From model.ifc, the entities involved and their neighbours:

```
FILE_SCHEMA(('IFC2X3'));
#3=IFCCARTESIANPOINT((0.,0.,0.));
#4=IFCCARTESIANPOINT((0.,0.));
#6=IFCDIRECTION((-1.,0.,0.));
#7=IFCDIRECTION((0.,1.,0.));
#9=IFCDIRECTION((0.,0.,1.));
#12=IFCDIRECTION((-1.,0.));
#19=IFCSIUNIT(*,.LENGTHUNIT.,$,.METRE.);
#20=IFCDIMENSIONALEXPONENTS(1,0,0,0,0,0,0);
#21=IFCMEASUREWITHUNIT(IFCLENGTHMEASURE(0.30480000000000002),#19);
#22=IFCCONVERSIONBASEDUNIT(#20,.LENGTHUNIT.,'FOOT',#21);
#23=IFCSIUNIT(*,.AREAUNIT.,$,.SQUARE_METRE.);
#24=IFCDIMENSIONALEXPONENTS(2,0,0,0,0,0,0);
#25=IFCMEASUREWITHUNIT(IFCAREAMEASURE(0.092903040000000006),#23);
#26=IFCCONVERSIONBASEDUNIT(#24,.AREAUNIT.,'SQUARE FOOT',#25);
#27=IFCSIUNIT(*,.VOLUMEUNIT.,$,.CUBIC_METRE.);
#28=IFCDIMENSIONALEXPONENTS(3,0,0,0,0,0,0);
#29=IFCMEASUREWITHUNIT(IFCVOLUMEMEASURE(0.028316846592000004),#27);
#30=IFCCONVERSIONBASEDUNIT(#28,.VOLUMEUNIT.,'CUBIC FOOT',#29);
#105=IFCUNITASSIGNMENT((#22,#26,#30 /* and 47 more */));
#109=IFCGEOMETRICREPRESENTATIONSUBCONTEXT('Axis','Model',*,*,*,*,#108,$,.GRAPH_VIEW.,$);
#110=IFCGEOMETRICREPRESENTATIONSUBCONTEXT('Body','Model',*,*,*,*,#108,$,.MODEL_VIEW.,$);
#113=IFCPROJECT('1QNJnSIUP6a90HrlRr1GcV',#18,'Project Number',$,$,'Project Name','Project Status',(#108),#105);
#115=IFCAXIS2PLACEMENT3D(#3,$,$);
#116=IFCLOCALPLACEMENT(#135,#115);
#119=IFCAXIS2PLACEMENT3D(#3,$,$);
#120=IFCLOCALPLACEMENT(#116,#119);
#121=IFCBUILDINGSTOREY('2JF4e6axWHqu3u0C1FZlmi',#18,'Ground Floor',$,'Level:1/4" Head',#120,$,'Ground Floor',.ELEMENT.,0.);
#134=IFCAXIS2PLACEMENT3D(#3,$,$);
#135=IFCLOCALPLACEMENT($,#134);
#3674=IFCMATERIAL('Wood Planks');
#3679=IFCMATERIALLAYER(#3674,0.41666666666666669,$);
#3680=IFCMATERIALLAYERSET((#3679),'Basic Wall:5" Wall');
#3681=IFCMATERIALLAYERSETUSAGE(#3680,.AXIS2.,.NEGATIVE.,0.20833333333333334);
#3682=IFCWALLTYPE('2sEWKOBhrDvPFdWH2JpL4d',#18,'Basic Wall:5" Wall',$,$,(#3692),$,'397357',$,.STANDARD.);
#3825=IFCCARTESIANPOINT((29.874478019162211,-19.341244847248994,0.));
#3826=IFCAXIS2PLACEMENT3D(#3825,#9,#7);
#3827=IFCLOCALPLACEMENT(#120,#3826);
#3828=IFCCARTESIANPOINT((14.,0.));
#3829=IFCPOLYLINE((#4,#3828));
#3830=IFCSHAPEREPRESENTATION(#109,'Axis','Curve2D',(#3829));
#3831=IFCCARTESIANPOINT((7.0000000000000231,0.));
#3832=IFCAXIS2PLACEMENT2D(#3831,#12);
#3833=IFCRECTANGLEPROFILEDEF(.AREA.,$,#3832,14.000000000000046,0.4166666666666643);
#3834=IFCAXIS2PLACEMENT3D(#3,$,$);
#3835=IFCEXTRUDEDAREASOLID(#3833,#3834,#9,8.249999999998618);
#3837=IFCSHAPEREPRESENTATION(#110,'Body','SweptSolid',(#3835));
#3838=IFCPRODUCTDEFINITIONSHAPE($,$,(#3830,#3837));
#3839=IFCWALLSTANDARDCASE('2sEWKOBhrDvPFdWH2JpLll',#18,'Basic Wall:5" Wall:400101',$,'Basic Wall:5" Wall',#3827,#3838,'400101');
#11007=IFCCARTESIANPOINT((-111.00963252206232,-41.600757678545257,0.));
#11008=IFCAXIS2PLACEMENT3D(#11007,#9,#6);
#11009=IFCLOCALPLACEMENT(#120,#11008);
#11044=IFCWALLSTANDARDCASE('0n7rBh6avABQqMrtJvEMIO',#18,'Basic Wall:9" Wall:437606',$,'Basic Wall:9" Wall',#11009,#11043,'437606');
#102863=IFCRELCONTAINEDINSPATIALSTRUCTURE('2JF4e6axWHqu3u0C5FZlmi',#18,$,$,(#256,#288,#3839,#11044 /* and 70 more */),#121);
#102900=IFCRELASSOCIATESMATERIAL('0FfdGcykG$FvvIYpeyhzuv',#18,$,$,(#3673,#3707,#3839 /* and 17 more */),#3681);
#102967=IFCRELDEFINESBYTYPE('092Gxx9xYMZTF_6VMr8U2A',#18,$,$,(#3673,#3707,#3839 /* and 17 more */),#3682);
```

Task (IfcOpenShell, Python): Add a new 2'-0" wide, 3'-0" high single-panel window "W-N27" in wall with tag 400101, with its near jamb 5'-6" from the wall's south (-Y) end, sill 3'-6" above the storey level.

```python
import numpy as np
import ifcopenshell
import ifcopenshell.api.feature
import ifcopenshell.api.geometry
import ifcopenshell.api.root
import ifcopenshell.api.spatial
import ifcopenshell.api.type
import ifcopenshell.geom
import ifcopenshell.util.element
import ifcopenshell.util.placement
import ifcopenshell.util.representation
import ifcopenshell.util.shape
import ifcopenshell.util.unit

model = ifcopenshell.open("model.ifc")
unit_scale = ifcopenshell.util.unit.calculate_unit_scale(model)
settings = ifcopenshell.geom.settings()


def volume(element):
    """Net volume in cubic metres, openings subtracted."""
    shape = ifcopenshell.geom.create_shape(settings, element)
    return ifcopenshell.util.shape.get_volume(shape.geometry)


wall = model.by_id(3839)
storey = ifcopenshell.util.element.get_container(wall, ifc_class="IfcBuildingStorey")
context = ifcopenshell.util.representation.get_context(model, "Model", "Body", "MODEL_VIEW")
before = volume(wall)

width, height, from_end, sill = 0.6096, 0.9144, 1.6764, 1.0668  # metres

# The wall runs along its own X axis, and the end named is its -X end.
wall_shape = ifcopenshell.geom.create_shape(settings, wall)
x, y, z = ifcopenshell.util.shape.get_vertices(wall_shape.geometry).T
start = x.min() + from_end
face, thickness = float(y.min()), float(y.max() - y.min())
wall_matrix = ifcopenshell.util.placement.get_local_placement(wall.ObjectPlacement)
level = ifcopenshell.util.placement.get_local_placement(storey.ObjectPlacement)[2, 3]


def in_wall(x, y):
    """Placement at x, y metres in the wall's axes, at sill height."""
    matrix = wall_matrix.copy()
    matrix[:, 3] = wall_matrix @ np.array([x / unit_scale, y / unit_scale, 0.0, 1.0])
    matrix[2, 3] = level + sill / unit_scale
    return matrix


# Opening: a box that overshoots both wall faces by 50 mm.
opening = ifcopenshell.api.root.create_entity(model, ifc_class="IfcOpeningElement")
box = ifcopenshell.api.geometry.add_wall_representation(
    model, context=context, length=width, height=height, thickness=thickness + 0.1
)
ifcopenshell.api.geometry.assign_representation(model, product=opening, representation=box)
ifcopenshell.api.geometry.edit_object_placement(model, product=opening, matrix=in_wall(start, face - 0.05), is_si=False)
ifcopenshell.api.feature.add_feature(model, feature=opening, element=wall)

window = ifcopenshell.api.root.create_entity(model, ifc_class="IfcWindow", name="W-N27")
window.OverallWidth, window.OverallHeight = width / unit_scale, height / unit_scale
body = ifcopenshell.api.geometry.add_window_representation(
    model,
    context=context,
    overall_width=window.OverallWidth,
    overall_height=window.OverallHeight,
    partition_type="SINGLE_PANEL",
)
ifcopenshell.api.geometry.assign_representation(model, product=window, representation=body)
ifcopenshell.api.spatial.assign_container(model, products=[window], relating_structure=storey)
fills = ifcopenshell.api.feature.add_filling(model, opening=opening, element=window)
fills.OwnerHistory = window.OwnerHistory  # required in IFC2X3

# IFC2X3 keeps the operation on the window style.
style = ifcopenshell.api.root.create_entity(model, ifc_class="IfcWindowStyle", name="W-N27")
style.OperationType, style.ConstructionType = "SINGLE_PANEL", "NOTDEFINED"
style.ParameterTakesPrecedence = style.Sizeable = False
ifcopenshell.api.type.assign_type(model, related_objects=[window], relating_type=style)

# Centre the window in the wall's thickness.
ifcopenshell.api.geometry.edit_object_placement(model, product=window, matrix=in_wall(start, face), is_si=False)
window_shape = ifcopenshell.geom.create_shape(settings, window)
depth = ifcopenshell.util.shape.get_vertices(window_shape.geometry)[:, 1]
offset = face + thickness / 2 - (depth.min() + depth.max()) / 2
ifcopenshell.api.geometry.edit_object_placement(model, product=window, matrix=in_wall(start, offset), is_si=False)

after = volume(wall)

print(f"wall volume {before:.3f} -> {after:.3f} m3")

model.write("model_edited.ifc")
```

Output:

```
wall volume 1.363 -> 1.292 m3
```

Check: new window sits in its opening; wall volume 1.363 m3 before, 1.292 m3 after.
